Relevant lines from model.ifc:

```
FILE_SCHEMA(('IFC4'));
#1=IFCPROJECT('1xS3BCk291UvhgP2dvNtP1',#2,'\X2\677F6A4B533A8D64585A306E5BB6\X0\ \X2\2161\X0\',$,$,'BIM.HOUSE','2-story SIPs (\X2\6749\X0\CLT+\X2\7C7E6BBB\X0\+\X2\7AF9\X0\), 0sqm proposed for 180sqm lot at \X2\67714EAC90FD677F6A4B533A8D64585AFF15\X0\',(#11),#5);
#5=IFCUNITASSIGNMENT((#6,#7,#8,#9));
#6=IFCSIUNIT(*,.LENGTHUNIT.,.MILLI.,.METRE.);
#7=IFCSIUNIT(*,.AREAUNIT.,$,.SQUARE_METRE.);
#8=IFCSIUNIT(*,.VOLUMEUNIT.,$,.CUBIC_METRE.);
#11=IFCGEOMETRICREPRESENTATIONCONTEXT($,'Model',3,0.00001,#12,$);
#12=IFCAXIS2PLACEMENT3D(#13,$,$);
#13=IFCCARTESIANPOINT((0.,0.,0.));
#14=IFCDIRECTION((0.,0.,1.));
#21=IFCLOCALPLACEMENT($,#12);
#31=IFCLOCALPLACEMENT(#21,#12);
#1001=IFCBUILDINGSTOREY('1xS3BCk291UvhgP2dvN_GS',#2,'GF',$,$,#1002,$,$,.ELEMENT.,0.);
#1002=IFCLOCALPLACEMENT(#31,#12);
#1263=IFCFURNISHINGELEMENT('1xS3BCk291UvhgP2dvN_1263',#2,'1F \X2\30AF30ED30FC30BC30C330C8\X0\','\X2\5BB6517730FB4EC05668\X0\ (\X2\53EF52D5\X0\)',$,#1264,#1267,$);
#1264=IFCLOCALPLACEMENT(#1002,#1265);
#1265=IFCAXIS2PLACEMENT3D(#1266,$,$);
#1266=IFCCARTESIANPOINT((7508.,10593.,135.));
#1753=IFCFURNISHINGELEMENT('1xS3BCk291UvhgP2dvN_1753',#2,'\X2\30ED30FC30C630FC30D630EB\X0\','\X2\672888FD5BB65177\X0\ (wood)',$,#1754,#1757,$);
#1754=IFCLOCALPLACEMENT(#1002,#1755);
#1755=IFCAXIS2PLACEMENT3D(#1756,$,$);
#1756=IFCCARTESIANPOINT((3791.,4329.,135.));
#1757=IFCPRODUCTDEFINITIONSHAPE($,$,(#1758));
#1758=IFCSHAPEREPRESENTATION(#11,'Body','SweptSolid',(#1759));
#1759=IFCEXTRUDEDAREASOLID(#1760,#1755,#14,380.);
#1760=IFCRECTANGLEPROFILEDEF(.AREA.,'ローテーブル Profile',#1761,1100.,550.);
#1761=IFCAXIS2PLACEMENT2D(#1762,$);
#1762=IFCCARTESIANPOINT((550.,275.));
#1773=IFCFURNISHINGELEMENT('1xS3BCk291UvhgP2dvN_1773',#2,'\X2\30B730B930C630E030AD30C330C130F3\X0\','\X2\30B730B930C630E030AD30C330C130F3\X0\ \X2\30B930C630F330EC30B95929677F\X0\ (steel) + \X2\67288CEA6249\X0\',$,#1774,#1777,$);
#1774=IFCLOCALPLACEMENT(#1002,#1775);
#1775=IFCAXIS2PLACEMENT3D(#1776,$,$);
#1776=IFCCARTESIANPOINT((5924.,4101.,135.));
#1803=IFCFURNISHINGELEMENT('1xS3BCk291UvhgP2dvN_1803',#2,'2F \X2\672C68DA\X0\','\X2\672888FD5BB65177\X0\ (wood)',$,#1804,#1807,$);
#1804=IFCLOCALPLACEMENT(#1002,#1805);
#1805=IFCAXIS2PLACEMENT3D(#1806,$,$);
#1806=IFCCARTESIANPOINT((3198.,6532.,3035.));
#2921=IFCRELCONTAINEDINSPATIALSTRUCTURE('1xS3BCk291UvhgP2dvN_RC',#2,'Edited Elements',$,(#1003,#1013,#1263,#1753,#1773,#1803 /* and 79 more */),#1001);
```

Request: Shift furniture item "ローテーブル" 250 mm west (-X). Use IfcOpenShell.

```python
import ifcopenshell
import ifcopenshell.api.geometry
import ifcopenshell.util.placement
import ifcopenshell.util.unit

model = ifcopenshell.open("model.ifc")
unit_scale = ifcopenshell.util.unit.calculate_unit_scale(model)

item = model.by_guid("1xS3BCk291UvhgP2dvN_1753")
matrix = ifcopenshell.util.placement.get_local_placement(item.ObjectPlacement)
matrix[0, 3] -= 0.25 / unit_scale
ifcopenshell.api.geometry.edit_object_placement(model, product=item, matrix=matrix, is_si=False)

print(ifcopenshell.util.placement.get_local_placement(item.ObjectPlacement).round(3) + 0.0)

model.write("model_v2.ifc")
```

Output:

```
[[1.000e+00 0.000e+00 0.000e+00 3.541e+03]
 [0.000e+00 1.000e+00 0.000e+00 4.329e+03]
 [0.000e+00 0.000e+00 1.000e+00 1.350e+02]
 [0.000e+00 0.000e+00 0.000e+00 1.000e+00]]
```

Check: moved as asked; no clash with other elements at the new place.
